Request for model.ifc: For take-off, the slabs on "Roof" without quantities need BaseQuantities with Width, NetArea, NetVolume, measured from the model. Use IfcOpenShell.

First a look at what the model holds.

```python
import ifcopenshell
import ifcopenshell.util.element
import ifcopenshell.util.unit

model = ifcopenshell.open("model.ifc")
print(model.schema)
for unit_type in ("LENGTHUNIT", "AREAUNIT", "VOLUMEUNIT"):
    print(unit_type, ifcopenshell.util.unit.calculate_unit_scale(model, unit_type))
storey = next(s for s in model.by_type("IfcBuildingStorey") if s.Name == "Roof")
slabs = [e for e in ifcopenshell.util.element.get_decomposition(storey) if e.is_a("IfcSlab")]
for e in sorted(slabs, key=lambda e: e.id()):
    print(e.id(), e.is_a(), e.Name, list(ifcopenshell.util.element.get_psets(e, qtos_only=True)), sep=" | ")
```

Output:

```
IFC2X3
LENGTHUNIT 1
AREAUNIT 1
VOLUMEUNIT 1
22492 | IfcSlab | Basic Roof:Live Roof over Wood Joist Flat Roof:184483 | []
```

```python
import ifcopenshell
import ifcopenshell.api.pset
import ifcopenshell.geom
import ifcopenshell.util.element
import ifcopenshell.util.shape
import ifcopenshell.util.unit

model = ifcopenshell.open("model.ifc")
unit_scale = ifcopenshell.util.unit.calculate_unit_scale(model)
area_scale = ifcopenshell.util.unit.calculate_unit_scale(model, "AREAUNIT")
volume_scale = ifcopenshell.util.unit.calculate_unit_scale(model, "VOLUMEUNIT")
settings = ifcopenshell.geom.settings()

storey = next(s for s in model.by_type("IfcBuildingStorey") if s.Name == "Roof")
slabs = [e for e in ifcopenshell.util.element.get_decomposition(storey) if e.is_a("IfcSlab")]

for e in sorted(slabs, key=lambda e: e.id()):
    if ifcopenshell.util.element.get_psets(e, qtos_only=True, should_inherit=False):
        continue
    # Geometry comes back in metres, in the element's own axes.
    shape = ifcopenshell.geom.create_shape(settings, e)
    values = {
        "Width": ifcopenshell.util.shape.get_z(shape.geometry) / unit_scale,
        "NetArea": ifcopenshell.util.shape.get_footprint_area(shape.geometry) / area_scale,
        "NetVolume": ifcopenshell.util.shape.get_volume(shape.geometry) / volume_scale,
    }
    qto = ifcopenshell.api.pset.add_qto(model, product=e, name="BaseQuantities")
    ifcopenshell.api.pset.edit_qto(model, qto=qto, properties=values)
    print(e.id(), {k: round(v, 3) for k, v in values.items()})

model.write("model_v2.ifc")
```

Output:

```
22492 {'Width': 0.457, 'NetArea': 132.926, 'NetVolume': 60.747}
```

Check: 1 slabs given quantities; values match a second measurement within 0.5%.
